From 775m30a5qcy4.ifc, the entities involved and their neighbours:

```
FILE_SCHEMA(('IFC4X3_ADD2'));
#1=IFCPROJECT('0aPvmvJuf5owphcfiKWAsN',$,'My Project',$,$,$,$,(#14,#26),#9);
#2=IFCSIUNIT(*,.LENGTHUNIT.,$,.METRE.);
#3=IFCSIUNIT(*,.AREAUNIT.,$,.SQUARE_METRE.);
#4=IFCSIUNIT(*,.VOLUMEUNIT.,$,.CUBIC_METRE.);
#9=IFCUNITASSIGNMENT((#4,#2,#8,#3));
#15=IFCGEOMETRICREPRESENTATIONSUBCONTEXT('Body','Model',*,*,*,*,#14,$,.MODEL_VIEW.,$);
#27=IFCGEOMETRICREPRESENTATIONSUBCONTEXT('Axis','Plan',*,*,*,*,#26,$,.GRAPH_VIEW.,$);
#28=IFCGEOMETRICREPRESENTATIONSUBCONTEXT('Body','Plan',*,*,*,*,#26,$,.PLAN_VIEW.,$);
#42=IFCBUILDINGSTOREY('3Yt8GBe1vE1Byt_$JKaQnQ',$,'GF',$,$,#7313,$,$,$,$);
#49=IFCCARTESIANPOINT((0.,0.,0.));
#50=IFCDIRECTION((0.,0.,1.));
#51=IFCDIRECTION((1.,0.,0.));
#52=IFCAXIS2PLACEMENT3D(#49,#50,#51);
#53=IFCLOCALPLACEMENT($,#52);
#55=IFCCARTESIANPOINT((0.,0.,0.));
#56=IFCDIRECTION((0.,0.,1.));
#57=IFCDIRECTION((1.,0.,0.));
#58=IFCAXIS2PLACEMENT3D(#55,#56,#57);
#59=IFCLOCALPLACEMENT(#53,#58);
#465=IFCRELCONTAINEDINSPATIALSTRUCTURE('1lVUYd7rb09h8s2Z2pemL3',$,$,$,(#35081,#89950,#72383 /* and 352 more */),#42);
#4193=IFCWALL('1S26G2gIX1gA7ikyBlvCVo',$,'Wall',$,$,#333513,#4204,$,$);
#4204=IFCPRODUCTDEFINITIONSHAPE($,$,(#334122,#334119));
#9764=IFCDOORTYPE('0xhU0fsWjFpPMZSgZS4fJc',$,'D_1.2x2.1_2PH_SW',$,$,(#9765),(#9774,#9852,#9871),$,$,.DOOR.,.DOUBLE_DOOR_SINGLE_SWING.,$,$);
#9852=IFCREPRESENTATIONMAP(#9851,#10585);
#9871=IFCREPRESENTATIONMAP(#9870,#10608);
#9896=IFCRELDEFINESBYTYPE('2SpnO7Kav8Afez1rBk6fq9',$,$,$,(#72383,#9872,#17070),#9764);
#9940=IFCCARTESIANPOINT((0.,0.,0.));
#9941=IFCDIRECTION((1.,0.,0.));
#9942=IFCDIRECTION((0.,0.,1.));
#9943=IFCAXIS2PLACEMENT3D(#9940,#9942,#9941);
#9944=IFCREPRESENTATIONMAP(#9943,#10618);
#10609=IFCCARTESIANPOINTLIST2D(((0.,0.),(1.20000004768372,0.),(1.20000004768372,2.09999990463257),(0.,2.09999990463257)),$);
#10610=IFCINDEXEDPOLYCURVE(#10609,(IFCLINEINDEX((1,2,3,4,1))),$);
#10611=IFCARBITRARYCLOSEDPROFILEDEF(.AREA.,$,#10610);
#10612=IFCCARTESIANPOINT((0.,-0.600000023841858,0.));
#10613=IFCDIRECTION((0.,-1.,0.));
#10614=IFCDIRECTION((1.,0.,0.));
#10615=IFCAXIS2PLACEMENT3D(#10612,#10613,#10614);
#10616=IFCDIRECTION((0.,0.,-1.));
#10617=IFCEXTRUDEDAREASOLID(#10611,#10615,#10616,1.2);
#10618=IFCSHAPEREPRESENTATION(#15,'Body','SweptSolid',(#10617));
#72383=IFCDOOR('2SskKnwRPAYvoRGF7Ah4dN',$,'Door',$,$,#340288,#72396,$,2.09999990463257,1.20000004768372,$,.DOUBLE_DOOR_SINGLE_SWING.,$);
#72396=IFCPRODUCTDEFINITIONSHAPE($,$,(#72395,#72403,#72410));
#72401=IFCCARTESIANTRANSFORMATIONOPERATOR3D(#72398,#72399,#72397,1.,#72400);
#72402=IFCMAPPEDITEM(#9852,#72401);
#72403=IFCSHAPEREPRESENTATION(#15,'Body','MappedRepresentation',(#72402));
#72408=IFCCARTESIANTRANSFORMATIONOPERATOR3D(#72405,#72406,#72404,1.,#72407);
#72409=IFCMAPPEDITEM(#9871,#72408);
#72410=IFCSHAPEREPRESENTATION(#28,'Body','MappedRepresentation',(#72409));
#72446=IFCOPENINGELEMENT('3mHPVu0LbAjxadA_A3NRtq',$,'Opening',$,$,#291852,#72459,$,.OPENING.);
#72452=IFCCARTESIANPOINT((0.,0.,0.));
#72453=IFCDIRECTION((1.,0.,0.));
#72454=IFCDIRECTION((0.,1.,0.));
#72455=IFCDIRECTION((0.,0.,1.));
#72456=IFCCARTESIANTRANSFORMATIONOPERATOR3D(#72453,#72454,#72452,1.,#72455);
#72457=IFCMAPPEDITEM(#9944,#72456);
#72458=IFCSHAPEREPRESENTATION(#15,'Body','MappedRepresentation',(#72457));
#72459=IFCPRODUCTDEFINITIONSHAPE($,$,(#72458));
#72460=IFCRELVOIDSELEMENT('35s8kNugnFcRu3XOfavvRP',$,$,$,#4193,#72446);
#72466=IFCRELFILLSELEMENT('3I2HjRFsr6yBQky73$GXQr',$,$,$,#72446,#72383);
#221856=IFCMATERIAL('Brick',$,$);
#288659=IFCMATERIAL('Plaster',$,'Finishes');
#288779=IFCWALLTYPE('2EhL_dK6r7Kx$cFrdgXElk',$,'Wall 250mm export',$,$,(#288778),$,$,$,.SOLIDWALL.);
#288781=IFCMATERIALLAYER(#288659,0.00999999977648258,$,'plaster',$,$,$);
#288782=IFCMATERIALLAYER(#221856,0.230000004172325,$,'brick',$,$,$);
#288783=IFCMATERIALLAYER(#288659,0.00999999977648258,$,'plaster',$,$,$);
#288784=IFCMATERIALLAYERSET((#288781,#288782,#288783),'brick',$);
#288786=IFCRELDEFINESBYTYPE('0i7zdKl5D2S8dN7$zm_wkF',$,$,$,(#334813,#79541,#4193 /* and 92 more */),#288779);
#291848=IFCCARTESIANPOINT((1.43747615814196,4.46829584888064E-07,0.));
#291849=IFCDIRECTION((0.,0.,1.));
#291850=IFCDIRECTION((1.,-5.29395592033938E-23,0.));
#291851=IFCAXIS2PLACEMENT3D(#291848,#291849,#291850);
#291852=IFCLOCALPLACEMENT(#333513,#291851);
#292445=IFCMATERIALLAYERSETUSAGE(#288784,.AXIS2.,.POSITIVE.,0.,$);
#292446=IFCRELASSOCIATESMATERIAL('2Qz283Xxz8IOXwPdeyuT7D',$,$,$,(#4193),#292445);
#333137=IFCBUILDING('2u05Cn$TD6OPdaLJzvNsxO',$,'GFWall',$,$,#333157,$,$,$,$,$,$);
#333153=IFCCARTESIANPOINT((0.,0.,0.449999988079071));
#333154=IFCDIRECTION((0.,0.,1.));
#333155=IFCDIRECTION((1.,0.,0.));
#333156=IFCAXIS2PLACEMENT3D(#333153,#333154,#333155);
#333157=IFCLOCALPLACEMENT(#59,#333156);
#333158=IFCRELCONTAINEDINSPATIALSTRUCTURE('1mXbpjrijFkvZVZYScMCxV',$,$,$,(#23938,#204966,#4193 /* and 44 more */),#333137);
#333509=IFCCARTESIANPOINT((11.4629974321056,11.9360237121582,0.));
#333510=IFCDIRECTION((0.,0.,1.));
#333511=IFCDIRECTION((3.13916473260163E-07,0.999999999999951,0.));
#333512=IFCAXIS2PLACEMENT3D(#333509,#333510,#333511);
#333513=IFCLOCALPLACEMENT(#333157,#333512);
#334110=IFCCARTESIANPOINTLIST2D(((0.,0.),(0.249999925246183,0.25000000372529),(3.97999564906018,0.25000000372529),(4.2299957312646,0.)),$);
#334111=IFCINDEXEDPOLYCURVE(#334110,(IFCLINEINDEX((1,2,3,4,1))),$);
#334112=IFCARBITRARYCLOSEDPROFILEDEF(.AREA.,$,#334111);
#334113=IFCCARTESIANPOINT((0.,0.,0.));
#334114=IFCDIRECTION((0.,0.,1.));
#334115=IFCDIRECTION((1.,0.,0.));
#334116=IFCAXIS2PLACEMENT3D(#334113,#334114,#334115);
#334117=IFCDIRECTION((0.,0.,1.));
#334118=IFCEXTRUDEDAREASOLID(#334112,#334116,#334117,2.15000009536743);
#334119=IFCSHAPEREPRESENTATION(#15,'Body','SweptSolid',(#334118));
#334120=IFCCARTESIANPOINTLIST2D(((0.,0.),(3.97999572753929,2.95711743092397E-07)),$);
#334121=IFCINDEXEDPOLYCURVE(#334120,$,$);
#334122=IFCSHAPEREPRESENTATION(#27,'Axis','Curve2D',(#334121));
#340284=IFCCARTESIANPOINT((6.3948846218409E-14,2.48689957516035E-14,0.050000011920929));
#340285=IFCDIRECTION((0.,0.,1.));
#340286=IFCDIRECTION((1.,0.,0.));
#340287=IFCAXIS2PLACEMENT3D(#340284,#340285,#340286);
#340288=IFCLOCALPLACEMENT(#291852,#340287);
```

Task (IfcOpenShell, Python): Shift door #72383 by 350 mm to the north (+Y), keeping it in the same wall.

```python
import ifcopenshell
import ifcopenshell.api.geometry
import ifcopenshell.util.placement

model = ifcopenshell.open("775m30a5qcy4.ifc")

door = model.by_guid("2SskKnwRPAYvoRGF7Ah4dN")
opening = door.FillsVoids[0].RelatingOpeningElement
wall = opening.VoidsElements[0].RelatingBuildingElement

wall_matrix = ifcopenshell.util.placement.get_local_placement(wall.ObjectPlacement)
shift = wall_matrix[:3, 0] * 0.35
before = ifcopenshell.util.placement.get_local_placement(door.ObjectPlacement)[:3, 3].copy()

# The door is placed relative to its opening, so it follows when the opening moves.
matrix = ifcopenshell.util.placement.get_local_placement(opening.ObjectPlacement)
matrix[:3, 3] += shift
ifcopenshell.api.geometry.edit_object_placement(
    model, product=opening, matrix=matrix, is_si=False, should_transform_children=True
)

after = ifcopenshell.util.placement.get_local_placement(door.ObjectPlacement)[:3, 3]
print("door moved by", (after - before).round(3) + 0.0)

model.write("775m30a5qcy4-out.ifc")
```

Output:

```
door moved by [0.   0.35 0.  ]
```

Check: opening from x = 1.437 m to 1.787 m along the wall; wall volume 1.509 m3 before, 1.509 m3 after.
